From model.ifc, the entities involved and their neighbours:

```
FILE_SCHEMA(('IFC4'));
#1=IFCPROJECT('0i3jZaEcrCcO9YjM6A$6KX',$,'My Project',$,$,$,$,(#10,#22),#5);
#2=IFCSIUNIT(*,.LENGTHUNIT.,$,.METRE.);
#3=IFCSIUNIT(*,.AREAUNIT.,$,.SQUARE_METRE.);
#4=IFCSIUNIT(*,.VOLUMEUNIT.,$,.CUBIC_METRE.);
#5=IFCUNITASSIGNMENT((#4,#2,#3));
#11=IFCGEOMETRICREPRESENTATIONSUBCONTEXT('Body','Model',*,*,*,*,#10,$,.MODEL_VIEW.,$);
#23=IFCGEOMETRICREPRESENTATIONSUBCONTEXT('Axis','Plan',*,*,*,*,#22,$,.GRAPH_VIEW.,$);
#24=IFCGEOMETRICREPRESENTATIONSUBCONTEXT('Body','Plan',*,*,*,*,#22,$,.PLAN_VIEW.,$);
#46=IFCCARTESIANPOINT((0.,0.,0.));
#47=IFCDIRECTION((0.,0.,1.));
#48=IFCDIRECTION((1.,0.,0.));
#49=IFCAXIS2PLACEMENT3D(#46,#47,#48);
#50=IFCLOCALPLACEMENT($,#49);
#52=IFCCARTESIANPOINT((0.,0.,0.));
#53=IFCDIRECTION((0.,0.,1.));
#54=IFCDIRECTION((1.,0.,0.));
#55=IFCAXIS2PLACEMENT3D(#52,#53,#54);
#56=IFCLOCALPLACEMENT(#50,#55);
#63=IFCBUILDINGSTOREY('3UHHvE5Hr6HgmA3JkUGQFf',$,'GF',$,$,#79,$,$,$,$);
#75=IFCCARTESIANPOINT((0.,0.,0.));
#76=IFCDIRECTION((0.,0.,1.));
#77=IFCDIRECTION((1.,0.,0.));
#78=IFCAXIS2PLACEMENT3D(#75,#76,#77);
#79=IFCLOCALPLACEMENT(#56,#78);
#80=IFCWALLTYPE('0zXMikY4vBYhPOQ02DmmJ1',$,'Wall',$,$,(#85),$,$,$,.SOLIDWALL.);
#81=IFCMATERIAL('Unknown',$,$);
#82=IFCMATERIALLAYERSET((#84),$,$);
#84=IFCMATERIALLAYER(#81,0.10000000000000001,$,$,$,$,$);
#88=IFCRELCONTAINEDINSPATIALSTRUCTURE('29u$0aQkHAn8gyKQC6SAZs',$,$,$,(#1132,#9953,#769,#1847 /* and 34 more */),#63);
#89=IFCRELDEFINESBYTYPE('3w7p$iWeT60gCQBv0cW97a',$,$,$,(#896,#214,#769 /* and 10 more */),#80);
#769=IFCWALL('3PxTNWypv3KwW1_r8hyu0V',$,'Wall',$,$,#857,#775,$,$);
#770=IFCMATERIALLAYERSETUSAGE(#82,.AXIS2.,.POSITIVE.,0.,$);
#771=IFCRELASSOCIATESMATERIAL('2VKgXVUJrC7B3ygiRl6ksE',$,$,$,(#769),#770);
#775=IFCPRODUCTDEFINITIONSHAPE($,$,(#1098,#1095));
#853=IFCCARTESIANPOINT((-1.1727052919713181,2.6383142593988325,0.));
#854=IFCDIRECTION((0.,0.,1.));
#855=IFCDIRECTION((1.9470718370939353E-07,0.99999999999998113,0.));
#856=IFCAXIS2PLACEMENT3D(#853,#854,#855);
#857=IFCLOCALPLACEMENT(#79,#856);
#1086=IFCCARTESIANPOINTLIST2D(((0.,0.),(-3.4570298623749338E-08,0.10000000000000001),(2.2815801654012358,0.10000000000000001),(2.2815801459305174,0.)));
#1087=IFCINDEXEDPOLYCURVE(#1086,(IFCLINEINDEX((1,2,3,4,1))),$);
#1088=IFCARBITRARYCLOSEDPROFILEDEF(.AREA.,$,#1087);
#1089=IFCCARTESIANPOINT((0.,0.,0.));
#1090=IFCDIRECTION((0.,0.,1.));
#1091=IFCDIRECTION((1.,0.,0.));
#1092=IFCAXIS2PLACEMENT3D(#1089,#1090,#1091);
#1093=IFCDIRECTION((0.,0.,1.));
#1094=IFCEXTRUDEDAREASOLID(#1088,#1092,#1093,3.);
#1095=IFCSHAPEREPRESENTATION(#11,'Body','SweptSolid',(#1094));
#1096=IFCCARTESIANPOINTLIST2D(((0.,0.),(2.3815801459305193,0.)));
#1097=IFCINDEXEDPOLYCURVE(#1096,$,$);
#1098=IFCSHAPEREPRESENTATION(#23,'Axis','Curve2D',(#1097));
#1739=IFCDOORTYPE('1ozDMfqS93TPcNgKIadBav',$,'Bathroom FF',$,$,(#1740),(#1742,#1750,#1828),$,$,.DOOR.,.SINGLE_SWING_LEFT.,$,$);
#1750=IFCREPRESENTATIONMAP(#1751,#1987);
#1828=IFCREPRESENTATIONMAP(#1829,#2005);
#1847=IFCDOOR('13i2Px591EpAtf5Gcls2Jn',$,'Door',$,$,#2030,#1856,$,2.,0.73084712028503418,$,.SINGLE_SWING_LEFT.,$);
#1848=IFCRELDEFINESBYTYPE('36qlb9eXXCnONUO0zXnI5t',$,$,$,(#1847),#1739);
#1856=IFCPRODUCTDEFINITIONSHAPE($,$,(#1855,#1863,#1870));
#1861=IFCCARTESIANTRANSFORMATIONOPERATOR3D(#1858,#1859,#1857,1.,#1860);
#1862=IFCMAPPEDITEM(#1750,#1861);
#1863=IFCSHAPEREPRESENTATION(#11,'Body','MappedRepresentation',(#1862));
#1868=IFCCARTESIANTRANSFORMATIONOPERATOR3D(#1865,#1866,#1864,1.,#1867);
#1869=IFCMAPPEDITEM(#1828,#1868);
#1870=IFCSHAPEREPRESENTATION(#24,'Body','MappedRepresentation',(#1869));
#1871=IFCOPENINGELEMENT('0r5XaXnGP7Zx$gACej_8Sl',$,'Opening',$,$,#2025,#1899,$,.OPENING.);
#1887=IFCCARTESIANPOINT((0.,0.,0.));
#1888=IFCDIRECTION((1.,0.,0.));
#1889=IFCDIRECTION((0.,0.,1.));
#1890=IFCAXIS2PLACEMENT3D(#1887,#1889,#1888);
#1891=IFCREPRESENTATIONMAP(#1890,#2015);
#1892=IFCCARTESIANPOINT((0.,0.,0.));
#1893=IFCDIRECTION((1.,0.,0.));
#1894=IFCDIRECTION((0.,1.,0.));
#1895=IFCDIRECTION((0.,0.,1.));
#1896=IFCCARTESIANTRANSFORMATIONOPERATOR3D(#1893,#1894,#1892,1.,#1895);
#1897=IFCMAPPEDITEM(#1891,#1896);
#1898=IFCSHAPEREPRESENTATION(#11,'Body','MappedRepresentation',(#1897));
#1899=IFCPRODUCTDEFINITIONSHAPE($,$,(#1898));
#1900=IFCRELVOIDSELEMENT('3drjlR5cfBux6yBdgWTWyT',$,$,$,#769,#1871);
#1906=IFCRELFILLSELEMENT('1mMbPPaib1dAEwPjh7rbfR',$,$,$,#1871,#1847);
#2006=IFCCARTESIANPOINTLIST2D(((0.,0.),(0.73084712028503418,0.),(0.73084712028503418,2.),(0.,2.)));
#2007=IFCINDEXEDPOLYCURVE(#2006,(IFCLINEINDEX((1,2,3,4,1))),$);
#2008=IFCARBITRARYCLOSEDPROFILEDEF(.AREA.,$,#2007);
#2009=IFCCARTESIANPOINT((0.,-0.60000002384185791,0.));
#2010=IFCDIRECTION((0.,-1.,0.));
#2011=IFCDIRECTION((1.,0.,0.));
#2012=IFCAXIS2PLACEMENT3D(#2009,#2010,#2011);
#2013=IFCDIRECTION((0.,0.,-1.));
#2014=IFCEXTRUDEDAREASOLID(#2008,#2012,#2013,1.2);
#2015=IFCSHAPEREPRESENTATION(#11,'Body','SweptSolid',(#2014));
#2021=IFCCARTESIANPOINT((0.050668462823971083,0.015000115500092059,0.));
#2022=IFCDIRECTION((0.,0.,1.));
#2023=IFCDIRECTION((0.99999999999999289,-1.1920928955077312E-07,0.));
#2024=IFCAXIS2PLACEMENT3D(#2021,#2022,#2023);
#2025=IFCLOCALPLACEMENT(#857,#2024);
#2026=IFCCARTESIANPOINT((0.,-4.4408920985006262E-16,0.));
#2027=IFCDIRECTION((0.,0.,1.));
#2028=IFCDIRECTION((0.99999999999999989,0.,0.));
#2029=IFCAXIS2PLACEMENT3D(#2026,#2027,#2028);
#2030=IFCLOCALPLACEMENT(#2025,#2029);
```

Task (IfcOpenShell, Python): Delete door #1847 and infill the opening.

```python
import ifcopenshell
import ifcopenshell.api.feature
import ifcopenshell.api.root
import ifcopenshell.geom
import ifcopenshell.util.shape

model = ifcopenshell.open("model.ifc")
settings = ifcopenshell.geom.settings()


def volume(element):
    """Net volume in cubic metres, openings subtracted."""
    shape = ifcopenshell.geom.create_shape(settings, element)
    return ifcopenshell.util.shape.get_volume(shape.geometry)


door = model.by_guid("13i2Px591EpAtf5Gcls2Jn")
opening = door.FillsVoids[0].RelatingOpeningElement
wall = opening.VoidsElements[0].RelatingBuildingElement
before = volume(wall)

ifcopenshell.api.root.remove_product(model, product=door)
ifcopenshell.api.feature.remove_feature(model, feature=opening)

after = volume(wall)

print(f"wall volume {before:.3f} -> {after:.3f} m3")

model.write("model_updated.ifc")
```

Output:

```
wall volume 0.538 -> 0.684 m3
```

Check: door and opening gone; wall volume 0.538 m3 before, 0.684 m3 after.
